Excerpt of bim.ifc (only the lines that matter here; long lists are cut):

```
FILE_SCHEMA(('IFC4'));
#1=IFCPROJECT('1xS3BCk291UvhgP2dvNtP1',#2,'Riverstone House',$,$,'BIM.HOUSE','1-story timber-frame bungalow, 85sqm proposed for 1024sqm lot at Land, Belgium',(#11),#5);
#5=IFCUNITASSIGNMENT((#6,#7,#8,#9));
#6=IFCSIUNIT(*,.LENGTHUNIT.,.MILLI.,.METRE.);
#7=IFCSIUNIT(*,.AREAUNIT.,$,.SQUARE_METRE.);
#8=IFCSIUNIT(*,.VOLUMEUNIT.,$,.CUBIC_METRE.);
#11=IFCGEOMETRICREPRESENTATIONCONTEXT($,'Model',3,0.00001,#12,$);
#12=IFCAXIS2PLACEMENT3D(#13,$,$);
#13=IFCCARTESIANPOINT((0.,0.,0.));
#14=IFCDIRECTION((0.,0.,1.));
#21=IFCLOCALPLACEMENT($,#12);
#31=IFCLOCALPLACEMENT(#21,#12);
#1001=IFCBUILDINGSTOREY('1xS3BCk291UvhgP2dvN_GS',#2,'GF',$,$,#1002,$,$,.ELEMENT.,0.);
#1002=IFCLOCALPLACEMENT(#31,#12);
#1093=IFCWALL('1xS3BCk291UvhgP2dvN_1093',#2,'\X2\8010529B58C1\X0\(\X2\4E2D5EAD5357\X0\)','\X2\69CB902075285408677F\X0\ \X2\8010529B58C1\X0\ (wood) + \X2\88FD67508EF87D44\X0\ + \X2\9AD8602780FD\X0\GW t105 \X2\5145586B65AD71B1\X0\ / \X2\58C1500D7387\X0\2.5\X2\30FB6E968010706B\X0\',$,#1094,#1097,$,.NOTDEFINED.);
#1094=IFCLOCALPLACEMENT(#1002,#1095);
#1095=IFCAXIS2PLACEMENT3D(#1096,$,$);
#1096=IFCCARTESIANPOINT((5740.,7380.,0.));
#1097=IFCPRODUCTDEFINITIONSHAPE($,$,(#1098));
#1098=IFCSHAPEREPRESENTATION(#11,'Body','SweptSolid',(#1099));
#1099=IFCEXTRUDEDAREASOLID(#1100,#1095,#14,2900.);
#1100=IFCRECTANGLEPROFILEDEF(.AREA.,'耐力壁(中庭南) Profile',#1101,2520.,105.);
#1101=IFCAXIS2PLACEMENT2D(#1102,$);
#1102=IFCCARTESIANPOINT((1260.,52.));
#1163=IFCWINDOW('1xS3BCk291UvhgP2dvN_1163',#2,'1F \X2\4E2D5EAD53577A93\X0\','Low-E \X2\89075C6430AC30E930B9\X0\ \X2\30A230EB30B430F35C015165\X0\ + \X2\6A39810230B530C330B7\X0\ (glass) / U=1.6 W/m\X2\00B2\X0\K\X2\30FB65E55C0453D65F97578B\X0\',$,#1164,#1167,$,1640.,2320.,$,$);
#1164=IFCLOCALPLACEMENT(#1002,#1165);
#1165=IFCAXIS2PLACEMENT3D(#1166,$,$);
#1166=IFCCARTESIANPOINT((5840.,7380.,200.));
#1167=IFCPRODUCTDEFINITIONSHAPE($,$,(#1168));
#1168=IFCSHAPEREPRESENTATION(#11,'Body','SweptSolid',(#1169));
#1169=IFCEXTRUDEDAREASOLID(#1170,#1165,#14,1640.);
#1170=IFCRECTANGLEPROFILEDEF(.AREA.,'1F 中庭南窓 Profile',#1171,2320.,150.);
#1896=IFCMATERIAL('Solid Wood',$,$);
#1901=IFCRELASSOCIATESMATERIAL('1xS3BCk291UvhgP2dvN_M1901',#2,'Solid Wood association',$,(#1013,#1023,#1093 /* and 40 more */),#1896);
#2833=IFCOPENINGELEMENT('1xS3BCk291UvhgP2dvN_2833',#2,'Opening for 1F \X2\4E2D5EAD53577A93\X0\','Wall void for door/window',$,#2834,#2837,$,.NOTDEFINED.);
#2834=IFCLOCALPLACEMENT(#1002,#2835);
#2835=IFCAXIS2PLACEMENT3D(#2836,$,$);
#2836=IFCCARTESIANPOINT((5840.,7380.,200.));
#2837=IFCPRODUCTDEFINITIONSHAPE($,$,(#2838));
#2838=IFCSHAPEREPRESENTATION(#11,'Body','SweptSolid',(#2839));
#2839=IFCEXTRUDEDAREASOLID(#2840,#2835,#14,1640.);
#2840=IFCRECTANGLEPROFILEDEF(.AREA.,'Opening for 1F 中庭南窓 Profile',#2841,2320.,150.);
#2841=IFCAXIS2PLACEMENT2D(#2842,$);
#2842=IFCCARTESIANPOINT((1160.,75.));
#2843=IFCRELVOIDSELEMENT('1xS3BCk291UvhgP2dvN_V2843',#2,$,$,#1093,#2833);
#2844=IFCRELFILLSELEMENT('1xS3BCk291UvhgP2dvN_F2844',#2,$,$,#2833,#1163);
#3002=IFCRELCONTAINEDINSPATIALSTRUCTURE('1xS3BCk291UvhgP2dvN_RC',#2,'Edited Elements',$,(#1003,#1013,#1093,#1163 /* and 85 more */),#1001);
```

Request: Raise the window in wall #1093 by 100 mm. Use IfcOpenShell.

```python
import numpy as np
import ifcopenshell
import ifcopenshell.api.geometry
import ifcopenshell.util.placement
import ifcopenshell.util.unit

model = ifcopenshell.open("bim.ifc")
unit_scale = ifcopenshell.util.unit.calculate_unit_scale(model)

window = model.by_guid("1xS3BCk291UvhgP2dvN_1163")
opening = window.FillsVoids[0].RelatingOpeningElement
dz = 0.1 / unit_scale

shift = np.array([0.0, 0.0, dz])
# The window is not placed relative to its opening, so move both.
for product in (opening, window):
    matrix = ifcopenshell.util.placement.get_local_placement(product.ObjectPlacement)
    matrix[:3, 3] += shift
    ifcopenshell.api.geometry.edit_object_placement(model, product=product, matrix=matrix, is_si=False)

print(f"moved by {dz * unit_scale:+.3f} m")

model.write("bim_v2.ifc")
```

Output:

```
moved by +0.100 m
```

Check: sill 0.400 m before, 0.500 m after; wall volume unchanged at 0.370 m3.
